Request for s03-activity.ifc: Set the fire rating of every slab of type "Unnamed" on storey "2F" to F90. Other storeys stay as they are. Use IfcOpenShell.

First a look at what the model holds.

```python
import ifcopenshell
import ifcopenshell.util.element

model = ifcopenshell.open("s03-activity.ifc")
print(model.schema)
storey = next(s for s in model.by_type("IfcBuildingStorey") if s.Name == "2F")
slabs = [e for e in ifcopenshell.util.element.get_decomposition(storey) if e.is_a("IfcSlab")]
seen = {}
for e in slabs:
    element_type = ifcopenshell.util.element.get_type(e)
    key = (element_type.Name if element_type != e and element_type else None, ifcopenshell.util.element.get_pset(e, "Pset_SlabCommon", "FireRating"))
    seen[key] = seen.get(key, 0) + 1
for (name, value), count in sorted(seen.items(), key=str):
    print(count, "x", name, "|", value)
```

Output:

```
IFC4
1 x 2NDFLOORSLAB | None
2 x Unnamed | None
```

```python
import ifcopenshell
import ifcopenshell.api.pset
import ifcopenshell.util.element

model = ifcopenshell.open("s03-activity.ifc")

storey = next(s for s in model.by_type("IfcBuildingStorey") if s.Name == "2F")
slabs = [e for e in ifcopenshell.util.element.get_decomposition(storey) if e.is_a("IfcSlab")]

count = 0
for e in slabs:
    element_type = ifcopenshell.util.element.get_type(e)
    if element_type in (None, e) or element_type.Name != "Unnamed":
        continue
    # add_pset returns the element's existing set when there is one.
    pset = ifcopenshell.api.pset.add_pset(model, product=e, name="Pset_SlabCommon")
    ifcopenshell.api.pset.edit_pset(model, pset=pset, properties={"FireRating": "F90"})
    count += 1

print(count, "slabs updated")

model.write("s03-activity_v2.ifc")
```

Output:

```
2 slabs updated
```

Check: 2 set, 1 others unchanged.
